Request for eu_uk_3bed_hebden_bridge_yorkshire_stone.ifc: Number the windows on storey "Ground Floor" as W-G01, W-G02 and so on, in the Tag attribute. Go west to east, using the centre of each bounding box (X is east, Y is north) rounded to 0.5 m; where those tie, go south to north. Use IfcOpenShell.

First a look at what the model holds.

```python
import ifcopenshell
import ifcopenshell.util.element
import ifcopenshell.util.placement

model = ifcopenshell.open("eu_uk_3bed_hebden_bridge_yorkshire_stone.ifc")
print(model.schema)
storey = next(s for s in model.by_type("IfcBuildingStorey") if s.Name == "Ground Floor")
windows = [e for e in ifcopenshell.util.element.get_decomposition(storey) if e.is_a("IfcWindow")]
for e in sorted(windows, key=lambda e: e.id()):
    origin = ifcopenshell.util.placement.get_local_placement(e.ObjectPlacement)[:3, 3]
    print(e.id(), e.Tag, e.Name, origin.round(2) + 0.0, sep=" | ")
```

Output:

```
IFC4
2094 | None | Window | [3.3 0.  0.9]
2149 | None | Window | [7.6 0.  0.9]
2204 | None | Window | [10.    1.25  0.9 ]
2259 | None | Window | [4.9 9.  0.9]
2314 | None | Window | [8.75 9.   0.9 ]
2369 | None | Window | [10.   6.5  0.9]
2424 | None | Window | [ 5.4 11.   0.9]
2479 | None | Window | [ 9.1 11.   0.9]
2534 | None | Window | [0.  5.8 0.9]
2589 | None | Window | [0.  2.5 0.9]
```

```python
import ifcopenshell
import ifcopenshell.geom
import ifcopenshell.util.element
import ifcopenshell.util.shape

model = ifcopenshell.open("eu_uk_3bed_hebden_bridge_yorkshire_stone.ifc")
settings = ifcopenshell.geom.settings()
settings.set("use-world-coords", True)


def centre(element):
    shape = ifcopenshell.geom.create_shape(settings, element)
    return ifcopenshell.util.shape.get_bbox_centroid(shape.geometry)


storey = next(s for s in model.by_type("IfcBuildingStorey") if s.Name == "Ground Floor")
windows = [e for e in ifcopenshell.util.element.get_decomposition(storey) if e.is_a("IfcWindow")]

# Insertion points can sit at a corner or the storey origin, so sort by the geometry (in metres).
centres = {e: centre(e) for e in windows}
windows.sort(key=lambda e: (round(centres[e][0] / 0.5), centres[e][1]))

for i, e in enumerate(windows, start=1):
    number = f"W-G{i:02d}"
    e.Tag = number
    print(e.id(), number)

model.write("eu_uk_3bed_hebden_bridge_yorkshire_stone_rev.ifc")
```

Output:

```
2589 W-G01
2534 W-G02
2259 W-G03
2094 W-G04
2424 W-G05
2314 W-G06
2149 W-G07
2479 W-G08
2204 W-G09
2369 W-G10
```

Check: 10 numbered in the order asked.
